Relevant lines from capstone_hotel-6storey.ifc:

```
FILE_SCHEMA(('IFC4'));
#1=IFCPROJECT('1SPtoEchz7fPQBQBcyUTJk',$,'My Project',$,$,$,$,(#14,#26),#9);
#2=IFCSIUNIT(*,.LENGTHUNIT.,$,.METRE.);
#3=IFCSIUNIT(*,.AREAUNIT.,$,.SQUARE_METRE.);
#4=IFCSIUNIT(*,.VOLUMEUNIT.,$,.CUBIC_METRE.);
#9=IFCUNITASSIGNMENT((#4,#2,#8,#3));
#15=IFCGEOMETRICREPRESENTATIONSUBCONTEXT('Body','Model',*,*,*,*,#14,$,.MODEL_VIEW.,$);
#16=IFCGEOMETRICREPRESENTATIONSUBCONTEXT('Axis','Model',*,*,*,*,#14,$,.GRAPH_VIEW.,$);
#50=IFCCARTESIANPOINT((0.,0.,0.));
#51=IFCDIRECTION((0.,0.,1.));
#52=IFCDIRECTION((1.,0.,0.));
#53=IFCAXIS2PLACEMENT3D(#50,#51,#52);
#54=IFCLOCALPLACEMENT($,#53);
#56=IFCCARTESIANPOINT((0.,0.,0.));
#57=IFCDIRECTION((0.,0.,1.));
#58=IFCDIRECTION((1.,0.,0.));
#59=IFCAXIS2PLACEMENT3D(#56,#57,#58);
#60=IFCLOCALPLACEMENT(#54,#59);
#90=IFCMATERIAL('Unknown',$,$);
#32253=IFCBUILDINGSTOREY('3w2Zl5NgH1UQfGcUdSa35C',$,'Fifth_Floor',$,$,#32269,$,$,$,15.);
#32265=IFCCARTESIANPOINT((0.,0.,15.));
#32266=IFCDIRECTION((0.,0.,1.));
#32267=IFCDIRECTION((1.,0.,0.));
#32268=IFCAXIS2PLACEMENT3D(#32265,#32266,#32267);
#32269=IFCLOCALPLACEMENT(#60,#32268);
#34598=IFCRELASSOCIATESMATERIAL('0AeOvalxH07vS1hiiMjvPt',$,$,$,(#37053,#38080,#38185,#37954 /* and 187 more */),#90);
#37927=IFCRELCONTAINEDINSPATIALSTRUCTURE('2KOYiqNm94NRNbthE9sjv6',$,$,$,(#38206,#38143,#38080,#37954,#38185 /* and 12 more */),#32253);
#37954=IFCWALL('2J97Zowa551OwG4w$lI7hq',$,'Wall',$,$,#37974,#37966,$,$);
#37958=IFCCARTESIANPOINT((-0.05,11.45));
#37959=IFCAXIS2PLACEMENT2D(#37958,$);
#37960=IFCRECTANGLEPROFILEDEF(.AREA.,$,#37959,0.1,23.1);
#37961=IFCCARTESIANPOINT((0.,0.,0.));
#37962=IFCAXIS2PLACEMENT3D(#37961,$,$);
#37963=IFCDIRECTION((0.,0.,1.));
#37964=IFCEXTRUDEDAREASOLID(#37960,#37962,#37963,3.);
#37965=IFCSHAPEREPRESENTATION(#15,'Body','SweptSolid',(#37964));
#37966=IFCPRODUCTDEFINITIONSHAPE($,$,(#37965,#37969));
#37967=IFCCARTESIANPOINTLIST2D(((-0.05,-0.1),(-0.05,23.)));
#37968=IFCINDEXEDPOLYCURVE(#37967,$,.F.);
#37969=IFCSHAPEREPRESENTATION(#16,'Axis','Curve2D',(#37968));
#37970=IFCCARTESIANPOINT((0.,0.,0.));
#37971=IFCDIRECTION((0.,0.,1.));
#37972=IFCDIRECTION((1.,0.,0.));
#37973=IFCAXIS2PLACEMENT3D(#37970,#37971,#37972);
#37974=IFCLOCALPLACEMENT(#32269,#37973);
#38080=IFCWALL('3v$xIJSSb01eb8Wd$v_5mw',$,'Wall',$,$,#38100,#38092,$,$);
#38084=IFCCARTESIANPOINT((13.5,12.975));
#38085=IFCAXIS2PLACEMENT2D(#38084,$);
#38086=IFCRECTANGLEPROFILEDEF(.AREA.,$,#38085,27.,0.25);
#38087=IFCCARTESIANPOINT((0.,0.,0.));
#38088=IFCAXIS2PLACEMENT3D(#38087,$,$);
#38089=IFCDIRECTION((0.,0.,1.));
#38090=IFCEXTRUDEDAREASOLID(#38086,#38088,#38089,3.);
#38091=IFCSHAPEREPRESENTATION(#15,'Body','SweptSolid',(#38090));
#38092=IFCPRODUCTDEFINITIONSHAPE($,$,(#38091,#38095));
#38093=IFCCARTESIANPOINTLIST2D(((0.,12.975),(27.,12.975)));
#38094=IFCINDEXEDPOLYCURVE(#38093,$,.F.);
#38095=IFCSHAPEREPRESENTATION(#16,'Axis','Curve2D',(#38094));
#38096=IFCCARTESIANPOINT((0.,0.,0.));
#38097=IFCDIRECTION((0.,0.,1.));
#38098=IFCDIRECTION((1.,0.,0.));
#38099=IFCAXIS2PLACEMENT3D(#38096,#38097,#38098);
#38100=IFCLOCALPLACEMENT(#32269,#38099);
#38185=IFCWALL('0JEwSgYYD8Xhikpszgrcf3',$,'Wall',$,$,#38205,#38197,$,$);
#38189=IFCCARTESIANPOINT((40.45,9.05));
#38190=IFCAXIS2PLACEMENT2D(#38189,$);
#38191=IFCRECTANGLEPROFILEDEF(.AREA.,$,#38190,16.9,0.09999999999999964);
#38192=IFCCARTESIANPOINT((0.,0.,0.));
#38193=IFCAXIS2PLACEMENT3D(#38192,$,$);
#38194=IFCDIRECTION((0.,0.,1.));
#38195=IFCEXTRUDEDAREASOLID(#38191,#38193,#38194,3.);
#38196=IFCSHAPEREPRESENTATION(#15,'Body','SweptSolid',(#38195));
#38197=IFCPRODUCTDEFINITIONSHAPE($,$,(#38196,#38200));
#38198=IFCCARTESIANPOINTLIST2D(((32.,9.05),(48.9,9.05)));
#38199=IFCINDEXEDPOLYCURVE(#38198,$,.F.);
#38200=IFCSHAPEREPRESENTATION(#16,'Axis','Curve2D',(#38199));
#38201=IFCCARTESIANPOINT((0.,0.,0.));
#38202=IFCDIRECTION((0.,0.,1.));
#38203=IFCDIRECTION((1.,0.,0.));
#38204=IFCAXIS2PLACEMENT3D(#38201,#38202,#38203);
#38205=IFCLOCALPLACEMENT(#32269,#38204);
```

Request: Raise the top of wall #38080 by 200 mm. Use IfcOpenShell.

```python
import ifcopenshell
import ifcopenshell.geom
import ifcopenshell.util.representation
import ifcopenshell.util.shape
import ifcopenshell.util.unit

model = ifcopenshell.open("capstone_hotel-6storey.ifc")
unit_scale = ifcopenshell.util.unit.calculate_unit_scale(model)
settings = ifcopenshell.geom.settings()


def volume(element):
    """Net volume in cubic metres, openings subtracted."""
    shape = ifcopenshell.geom.create_shape(settings, element)
    return ifcopenshell.util.shape.get_volume(shape.geometry)


wall = model.by_guid("3v$xIJSSb01eb8Wd$v_5mw")
before = volume(wall)

body = ifcopenshell.util.representation.get_representation(wall, "Model", "Body")
solid = body.Items[0]
old_height = solid.Depth
solid.Depth += 0.2 / unit_scale
after = volume(wall)

print(f"height {old_height:g} -> {solid.Depth:g}, volume {before:.3f} -> {after:.3f} m3")

model.write("capstone_hotel-6storey_edited.ifc")
```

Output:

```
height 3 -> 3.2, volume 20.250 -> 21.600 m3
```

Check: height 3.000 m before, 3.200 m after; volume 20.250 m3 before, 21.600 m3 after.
